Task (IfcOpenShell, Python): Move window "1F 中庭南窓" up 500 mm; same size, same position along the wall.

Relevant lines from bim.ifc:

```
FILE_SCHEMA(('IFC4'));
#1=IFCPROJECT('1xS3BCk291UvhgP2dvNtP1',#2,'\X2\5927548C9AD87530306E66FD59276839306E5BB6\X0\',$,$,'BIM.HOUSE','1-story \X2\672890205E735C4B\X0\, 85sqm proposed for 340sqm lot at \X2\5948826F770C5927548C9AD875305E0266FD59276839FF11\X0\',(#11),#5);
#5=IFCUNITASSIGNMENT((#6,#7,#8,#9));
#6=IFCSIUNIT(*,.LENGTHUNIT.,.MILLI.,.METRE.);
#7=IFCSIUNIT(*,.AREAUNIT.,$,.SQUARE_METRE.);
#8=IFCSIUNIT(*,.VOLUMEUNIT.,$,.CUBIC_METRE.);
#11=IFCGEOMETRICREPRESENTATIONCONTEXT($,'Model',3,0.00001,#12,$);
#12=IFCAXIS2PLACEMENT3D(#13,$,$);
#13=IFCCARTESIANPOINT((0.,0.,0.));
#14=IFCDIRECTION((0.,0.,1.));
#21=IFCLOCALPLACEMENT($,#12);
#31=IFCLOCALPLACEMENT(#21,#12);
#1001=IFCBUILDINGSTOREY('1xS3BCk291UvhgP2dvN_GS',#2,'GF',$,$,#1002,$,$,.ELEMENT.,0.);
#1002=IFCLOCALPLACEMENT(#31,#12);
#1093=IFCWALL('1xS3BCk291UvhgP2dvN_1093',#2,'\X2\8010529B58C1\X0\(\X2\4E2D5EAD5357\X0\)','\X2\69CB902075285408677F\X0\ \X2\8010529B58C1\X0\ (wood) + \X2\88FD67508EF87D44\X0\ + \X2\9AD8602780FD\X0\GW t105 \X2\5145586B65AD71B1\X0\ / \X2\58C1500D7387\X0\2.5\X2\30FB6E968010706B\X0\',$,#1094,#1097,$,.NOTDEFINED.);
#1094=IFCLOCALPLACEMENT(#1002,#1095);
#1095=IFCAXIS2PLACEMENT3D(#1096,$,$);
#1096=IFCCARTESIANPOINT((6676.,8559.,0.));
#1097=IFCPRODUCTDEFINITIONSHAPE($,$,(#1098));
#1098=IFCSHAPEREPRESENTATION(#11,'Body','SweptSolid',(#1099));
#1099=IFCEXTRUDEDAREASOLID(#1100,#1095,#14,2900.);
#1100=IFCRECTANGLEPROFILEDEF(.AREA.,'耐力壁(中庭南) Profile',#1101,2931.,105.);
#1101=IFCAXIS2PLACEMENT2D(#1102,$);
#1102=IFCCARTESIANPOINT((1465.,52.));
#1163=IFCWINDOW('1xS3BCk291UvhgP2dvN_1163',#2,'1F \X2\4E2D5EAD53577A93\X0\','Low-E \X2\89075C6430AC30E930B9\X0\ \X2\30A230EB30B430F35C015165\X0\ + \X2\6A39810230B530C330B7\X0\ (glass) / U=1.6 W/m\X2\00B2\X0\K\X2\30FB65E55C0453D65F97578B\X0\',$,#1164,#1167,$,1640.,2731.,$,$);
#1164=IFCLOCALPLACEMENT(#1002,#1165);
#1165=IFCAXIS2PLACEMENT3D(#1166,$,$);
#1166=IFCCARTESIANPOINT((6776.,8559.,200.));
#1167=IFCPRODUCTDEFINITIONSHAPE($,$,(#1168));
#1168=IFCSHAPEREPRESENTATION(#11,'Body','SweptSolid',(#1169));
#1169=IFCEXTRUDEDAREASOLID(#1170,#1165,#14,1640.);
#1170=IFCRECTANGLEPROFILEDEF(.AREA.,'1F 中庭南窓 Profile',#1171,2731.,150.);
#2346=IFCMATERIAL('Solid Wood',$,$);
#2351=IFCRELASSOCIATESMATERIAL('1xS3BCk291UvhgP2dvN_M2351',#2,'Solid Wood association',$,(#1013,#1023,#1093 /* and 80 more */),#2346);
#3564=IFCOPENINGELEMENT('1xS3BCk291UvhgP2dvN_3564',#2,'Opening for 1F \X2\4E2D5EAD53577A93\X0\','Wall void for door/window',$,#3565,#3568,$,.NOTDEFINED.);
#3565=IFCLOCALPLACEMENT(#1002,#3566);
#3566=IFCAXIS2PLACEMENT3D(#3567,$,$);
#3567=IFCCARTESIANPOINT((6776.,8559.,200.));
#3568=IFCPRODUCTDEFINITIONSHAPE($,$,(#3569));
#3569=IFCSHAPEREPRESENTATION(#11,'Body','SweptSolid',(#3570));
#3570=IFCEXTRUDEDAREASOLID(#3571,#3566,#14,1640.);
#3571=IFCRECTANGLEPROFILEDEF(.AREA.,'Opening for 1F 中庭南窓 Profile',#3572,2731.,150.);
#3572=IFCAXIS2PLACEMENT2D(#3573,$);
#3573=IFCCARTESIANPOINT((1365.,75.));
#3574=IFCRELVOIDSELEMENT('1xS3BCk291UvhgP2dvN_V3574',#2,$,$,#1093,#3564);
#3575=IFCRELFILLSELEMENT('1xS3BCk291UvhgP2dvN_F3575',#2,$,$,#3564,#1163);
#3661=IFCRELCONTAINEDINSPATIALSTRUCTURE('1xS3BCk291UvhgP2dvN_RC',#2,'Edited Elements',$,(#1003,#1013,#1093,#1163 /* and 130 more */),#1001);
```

```python
import numpy as np
import ifcopenshell
import ifcopenshell.api.geometry
import ifcopenshell.util.placement
import ifcopenshell.util.unit

model = ifcopenshell.open("bim.ifc")
unit_scale = ifcopenshell.util.unit.calculate_unit_scale(model)

window = model.by_id(1163)
opening = window.FillsVoids[0].RelatingOpeningElement
dz = 0.5 / unit_scale

shift = np.array([0.0, 0.0, dz])
# The window is not placed relative to its opening, so move both.
for product in (opening, window):
    matrix = ifcopenshell.util.placement.get_local_placement(product.ObjectPlacement)
    matrix[:3, 3] += shift
    ifcopenshell.api.geometry.edit_object_placement(model, product=product, matrix=matrix, is_si=False)

print(f"moved by {dz * unit_scale:+.3f} m")

model.write("bim_edited.ifc")
```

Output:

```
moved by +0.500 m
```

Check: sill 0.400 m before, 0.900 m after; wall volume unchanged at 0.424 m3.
